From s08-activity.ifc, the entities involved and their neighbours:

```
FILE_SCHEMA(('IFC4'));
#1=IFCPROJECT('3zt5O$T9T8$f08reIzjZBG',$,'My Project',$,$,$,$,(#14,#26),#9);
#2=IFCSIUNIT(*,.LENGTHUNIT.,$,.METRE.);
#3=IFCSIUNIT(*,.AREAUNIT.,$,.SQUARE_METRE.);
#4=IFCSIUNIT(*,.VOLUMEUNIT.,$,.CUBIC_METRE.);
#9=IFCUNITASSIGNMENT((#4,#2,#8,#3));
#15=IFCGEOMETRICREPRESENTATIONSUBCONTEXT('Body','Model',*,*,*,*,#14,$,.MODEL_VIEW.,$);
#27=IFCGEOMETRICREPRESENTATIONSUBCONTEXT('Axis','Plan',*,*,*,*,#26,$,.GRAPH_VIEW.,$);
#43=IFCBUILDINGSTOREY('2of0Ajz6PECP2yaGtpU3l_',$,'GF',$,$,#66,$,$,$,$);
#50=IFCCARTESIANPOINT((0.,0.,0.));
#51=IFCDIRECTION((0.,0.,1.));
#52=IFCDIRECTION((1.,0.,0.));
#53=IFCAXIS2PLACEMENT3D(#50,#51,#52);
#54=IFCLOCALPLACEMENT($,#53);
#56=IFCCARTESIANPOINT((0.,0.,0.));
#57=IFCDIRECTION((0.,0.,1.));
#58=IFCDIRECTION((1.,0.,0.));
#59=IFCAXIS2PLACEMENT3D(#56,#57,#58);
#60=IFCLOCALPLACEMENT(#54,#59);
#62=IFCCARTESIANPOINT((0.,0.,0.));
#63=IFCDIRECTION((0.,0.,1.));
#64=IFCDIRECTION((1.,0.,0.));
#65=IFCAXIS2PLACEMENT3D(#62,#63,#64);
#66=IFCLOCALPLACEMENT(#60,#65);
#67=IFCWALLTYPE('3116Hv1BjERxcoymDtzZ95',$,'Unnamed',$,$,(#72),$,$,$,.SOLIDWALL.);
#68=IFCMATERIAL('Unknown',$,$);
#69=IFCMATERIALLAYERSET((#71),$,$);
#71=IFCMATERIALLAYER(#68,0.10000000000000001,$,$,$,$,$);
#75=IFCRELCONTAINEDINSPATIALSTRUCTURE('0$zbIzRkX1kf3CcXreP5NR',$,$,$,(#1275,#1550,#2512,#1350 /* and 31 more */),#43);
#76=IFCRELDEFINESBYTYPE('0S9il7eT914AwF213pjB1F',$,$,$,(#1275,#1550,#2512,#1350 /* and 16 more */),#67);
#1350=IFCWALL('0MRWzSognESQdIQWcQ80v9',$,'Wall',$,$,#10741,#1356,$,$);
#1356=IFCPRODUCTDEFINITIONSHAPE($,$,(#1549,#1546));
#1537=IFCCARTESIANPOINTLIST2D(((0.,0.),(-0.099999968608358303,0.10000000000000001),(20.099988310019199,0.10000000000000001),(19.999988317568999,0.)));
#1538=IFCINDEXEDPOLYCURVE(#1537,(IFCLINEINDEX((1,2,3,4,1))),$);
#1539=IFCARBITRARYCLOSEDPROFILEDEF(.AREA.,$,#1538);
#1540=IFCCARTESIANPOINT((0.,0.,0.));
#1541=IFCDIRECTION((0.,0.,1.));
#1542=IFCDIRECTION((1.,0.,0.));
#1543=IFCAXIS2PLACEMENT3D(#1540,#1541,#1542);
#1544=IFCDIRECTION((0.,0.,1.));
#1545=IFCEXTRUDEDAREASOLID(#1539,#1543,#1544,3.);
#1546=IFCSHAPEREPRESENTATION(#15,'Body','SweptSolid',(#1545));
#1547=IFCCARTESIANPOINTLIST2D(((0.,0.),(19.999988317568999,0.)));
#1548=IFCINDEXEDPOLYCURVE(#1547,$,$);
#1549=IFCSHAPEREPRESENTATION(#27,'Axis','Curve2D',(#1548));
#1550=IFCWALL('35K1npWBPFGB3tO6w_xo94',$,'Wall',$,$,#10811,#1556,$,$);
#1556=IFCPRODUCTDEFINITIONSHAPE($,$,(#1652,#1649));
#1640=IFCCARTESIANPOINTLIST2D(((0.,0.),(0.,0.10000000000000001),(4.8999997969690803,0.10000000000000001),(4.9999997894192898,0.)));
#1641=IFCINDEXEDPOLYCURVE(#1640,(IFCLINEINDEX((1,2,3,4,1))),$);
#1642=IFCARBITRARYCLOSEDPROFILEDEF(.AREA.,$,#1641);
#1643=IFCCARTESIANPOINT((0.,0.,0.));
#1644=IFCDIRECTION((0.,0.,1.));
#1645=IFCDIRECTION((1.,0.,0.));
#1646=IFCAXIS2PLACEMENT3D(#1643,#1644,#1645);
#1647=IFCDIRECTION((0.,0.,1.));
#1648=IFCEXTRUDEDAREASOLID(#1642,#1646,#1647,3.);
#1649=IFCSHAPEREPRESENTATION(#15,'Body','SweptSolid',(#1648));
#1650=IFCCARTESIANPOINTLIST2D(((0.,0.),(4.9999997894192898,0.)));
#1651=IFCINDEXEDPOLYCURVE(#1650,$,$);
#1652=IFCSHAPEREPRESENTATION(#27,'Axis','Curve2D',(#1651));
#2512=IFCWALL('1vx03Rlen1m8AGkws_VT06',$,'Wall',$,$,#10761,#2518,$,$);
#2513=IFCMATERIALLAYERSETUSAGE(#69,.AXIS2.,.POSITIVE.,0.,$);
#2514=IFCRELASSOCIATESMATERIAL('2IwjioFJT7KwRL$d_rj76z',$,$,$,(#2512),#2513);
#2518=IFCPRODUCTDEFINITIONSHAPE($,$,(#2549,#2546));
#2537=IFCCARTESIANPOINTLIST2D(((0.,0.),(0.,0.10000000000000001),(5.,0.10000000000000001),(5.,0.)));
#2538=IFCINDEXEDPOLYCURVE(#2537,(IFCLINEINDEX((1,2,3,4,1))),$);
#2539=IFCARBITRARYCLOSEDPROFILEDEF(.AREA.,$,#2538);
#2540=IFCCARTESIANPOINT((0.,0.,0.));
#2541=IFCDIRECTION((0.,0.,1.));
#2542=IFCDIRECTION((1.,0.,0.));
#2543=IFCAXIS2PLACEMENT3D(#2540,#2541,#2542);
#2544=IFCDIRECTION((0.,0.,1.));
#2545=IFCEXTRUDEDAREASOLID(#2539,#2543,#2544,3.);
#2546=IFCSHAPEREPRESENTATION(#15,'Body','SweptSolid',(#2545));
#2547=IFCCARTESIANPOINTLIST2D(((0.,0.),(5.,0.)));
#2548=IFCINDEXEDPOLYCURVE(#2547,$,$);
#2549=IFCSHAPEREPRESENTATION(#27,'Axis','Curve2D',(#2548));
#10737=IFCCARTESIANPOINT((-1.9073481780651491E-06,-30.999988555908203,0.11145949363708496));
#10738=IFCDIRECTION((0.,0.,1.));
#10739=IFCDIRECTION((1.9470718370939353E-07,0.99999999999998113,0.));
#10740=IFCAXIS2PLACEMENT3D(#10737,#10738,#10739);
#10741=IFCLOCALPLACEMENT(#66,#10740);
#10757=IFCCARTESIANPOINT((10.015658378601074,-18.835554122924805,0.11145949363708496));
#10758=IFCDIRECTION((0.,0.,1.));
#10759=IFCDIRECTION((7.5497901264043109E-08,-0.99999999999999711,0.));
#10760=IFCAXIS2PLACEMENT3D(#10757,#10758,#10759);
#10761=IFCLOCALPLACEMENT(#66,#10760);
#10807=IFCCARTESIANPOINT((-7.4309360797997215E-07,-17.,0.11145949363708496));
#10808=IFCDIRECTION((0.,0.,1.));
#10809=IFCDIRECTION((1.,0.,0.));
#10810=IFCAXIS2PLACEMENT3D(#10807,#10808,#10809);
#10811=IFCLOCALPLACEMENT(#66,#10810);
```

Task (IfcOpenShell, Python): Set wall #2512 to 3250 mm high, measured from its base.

```python
import ifcopenshell
import ifcopenshell.geom
import ifcopenshell.util.representation
import ifcopenshell.util.shape

model = ifcopenshell.open("s08-activity.ifc")
settings = ifcopenshell.geom.settings()


def volume(element):
    """Net volume in cubic metres, openings subtracted."""
    shape = ifcopenshell.geom.create_shape(settings, element)
    return ifcopenshell.util.shape.get_volume(shape.geometry)


wall = model.by_id(2512)
before = volume(wall)

body = ifcopenshell.util.representation.get_representation(wall, "Model", "Body")
solid = body.Items[0]
old_height = solid.Depth
solid.Depth = 3.25
after = volume(wall)

print(f"height {old_height:g} -> {solid.Depth:g}, volume {before:.3f} -> {after:.3f} m3")

model.write("s08-activity_rev.ifc")
```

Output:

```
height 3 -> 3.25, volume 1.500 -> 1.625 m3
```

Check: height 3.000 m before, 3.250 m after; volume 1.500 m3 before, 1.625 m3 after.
